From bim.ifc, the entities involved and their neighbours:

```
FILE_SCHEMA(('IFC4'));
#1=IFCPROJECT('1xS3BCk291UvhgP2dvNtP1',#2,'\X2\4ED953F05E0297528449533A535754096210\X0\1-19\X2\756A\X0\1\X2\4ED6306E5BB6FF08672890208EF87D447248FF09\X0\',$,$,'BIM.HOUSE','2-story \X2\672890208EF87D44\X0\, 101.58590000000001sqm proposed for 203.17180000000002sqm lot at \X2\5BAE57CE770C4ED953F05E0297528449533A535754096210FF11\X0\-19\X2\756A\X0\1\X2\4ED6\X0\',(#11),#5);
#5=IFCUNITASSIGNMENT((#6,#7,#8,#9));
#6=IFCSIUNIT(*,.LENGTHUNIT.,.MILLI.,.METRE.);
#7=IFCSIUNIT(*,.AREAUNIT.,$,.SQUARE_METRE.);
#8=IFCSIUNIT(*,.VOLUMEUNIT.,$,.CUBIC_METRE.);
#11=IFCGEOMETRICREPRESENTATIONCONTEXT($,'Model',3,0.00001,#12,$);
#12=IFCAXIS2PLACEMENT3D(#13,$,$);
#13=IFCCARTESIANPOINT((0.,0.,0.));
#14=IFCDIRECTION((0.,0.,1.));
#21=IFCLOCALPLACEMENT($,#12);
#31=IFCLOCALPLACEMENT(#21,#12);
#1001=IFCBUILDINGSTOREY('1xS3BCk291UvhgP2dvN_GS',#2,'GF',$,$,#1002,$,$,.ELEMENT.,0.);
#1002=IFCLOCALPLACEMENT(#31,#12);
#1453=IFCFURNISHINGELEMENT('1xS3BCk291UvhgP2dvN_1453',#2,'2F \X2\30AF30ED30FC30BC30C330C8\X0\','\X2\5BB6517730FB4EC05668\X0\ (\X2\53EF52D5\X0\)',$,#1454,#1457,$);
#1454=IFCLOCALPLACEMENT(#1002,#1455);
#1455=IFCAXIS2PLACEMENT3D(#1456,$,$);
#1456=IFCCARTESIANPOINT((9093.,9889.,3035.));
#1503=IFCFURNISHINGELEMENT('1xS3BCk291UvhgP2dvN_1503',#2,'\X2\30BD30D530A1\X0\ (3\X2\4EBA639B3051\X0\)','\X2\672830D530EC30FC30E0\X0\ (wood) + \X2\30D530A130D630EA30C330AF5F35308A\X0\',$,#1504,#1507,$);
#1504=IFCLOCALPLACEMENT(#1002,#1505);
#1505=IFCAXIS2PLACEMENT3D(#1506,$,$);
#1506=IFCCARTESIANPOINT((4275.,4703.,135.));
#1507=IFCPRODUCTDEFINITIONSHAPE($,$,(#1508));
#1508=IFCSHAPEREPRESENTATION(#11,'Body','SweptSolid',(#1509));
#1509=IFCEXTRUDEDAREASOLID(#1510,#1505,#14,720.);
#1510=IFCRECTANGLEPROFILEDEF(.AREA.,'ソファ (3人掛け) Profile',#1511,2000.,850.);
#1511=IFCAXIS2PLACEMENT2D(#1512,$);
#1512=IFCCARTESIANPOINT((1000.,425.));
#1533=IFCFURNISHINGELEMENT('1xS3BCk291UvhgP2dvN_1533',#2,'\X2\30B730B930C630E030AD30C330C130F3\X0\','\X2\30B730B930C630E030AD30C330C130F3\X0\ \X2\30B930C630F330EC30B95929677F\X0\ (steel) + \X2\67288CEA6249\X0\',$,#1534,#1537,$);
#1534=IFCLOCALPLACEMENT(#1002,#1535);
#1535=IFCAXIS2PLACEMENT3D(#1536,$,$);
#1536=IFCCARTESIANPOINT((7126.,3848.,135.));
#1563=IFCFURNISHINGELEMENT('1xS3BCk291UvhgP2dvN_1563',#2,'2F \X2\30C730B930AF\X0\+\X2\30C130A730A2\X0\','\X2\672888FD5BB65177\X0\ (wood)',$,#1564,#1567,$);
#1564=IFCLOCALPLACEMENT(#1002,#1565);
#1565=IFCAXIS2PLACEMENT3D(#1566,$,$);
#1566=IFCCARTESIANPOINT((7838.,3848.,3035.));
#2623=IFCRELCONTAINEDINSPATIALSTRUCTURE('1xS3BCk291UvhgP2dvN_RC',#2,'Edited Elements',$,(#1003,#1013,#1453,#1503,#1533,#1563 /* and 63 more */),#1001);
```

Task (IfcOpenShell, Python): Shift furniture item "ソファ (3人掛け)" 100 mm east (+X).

```python
import ifcopenshell
import ifcopenshell.api.geometry
import ifcopenshell.util.placement

model = ifcopenshell.open("bim.ifc")

item = model.by_guid("1xS3BCk291UvhgP2dvN_1503")
matrix = ifcopenshell.util.placement.get_local_placement(item.ObjectPlacement)
matrix[0, 3] += 100.0
ifcopenshell.api.geometry.edit_object_placement(model, product=item, matrix=matrix, is_si=False)

print(ifcopenshell.util.placement.get_local_placement(item.ObjectPlacement).round(3) + 0.0)

model.write("bim_edited.ifc")
```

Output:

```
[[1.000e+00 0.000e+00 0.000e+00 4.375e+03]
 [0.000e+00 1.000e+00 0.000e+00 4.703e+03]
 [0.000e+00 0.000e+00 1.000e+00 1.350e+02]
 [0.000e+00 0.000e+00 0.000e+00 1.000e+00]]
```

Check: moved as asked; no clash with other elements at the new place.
